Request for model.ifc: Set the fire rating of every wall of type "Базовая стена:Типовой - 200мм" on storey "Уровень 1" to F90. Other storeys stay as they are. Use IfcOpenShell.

First a look at what the model holds.

```python
import ifcopenshell
import ifcopenshell.util.element

model = ifcopenshell.open("model.ifc")
print(model.schema)
storey = next(s for s in model.by_type("IfcBuildingStorey") if s.Name == "Уровень 1")
walls = [e for e in ifcopenshell.util.element.get_decomposition(storey) if e.is_a("IfcWall")]
seen = {}
for e in walls:
    element_type = ifcopenshell.util.element.get_type(e)
    key = (element_type.Name if element_type != e and element_type else None, ifcopenshell.util.element.get_pset(e, "Pset_WallCommon", "FireRating"))
    seen[key] = seen.get(key, 0) + 1
for (name, value), count in sorted(seen.items(), key=str):
    print(count, "x", name, "|", value)
```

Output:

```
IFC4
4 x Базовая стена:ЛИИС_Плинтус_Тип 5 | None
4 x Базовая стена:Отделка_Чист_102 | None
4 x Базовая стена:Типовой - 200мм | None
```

```python
import ifcopenshell
import ifcopenshell.api.pset
import ifcopenshell.util.element

model = ifcopenshell.open("model.ifc")

storey = next(s for s in model.by_type("IfcBuildingStorey") if s.Name == "Уровень 1")
walls = [e for e in ifcopenshell.util.element.get_decomposition(storey) if e.is_a("IfcWall")]

count = 0
for e in walls:
    element_type = ifcopenshell.util.element.get_type(e)
    if element_type in (None, e) or element_type.Name != "Базовая стена:Типовой - 200мм":
        continue
    # add_pset returns the element's existing set when there is one.
    pset = ifcopenshell.api.pset.add_pset(model, product=e, name="Pset_WallCommon")
    ifcopenshell.api.pset.edit_pset(model, pset=pset, properties={"FireRating": "F90"})
    count += 1

print(count, "walls updated")

model.write("model_edited.ifc")
```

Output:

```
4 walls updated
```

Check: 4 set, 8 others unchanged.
